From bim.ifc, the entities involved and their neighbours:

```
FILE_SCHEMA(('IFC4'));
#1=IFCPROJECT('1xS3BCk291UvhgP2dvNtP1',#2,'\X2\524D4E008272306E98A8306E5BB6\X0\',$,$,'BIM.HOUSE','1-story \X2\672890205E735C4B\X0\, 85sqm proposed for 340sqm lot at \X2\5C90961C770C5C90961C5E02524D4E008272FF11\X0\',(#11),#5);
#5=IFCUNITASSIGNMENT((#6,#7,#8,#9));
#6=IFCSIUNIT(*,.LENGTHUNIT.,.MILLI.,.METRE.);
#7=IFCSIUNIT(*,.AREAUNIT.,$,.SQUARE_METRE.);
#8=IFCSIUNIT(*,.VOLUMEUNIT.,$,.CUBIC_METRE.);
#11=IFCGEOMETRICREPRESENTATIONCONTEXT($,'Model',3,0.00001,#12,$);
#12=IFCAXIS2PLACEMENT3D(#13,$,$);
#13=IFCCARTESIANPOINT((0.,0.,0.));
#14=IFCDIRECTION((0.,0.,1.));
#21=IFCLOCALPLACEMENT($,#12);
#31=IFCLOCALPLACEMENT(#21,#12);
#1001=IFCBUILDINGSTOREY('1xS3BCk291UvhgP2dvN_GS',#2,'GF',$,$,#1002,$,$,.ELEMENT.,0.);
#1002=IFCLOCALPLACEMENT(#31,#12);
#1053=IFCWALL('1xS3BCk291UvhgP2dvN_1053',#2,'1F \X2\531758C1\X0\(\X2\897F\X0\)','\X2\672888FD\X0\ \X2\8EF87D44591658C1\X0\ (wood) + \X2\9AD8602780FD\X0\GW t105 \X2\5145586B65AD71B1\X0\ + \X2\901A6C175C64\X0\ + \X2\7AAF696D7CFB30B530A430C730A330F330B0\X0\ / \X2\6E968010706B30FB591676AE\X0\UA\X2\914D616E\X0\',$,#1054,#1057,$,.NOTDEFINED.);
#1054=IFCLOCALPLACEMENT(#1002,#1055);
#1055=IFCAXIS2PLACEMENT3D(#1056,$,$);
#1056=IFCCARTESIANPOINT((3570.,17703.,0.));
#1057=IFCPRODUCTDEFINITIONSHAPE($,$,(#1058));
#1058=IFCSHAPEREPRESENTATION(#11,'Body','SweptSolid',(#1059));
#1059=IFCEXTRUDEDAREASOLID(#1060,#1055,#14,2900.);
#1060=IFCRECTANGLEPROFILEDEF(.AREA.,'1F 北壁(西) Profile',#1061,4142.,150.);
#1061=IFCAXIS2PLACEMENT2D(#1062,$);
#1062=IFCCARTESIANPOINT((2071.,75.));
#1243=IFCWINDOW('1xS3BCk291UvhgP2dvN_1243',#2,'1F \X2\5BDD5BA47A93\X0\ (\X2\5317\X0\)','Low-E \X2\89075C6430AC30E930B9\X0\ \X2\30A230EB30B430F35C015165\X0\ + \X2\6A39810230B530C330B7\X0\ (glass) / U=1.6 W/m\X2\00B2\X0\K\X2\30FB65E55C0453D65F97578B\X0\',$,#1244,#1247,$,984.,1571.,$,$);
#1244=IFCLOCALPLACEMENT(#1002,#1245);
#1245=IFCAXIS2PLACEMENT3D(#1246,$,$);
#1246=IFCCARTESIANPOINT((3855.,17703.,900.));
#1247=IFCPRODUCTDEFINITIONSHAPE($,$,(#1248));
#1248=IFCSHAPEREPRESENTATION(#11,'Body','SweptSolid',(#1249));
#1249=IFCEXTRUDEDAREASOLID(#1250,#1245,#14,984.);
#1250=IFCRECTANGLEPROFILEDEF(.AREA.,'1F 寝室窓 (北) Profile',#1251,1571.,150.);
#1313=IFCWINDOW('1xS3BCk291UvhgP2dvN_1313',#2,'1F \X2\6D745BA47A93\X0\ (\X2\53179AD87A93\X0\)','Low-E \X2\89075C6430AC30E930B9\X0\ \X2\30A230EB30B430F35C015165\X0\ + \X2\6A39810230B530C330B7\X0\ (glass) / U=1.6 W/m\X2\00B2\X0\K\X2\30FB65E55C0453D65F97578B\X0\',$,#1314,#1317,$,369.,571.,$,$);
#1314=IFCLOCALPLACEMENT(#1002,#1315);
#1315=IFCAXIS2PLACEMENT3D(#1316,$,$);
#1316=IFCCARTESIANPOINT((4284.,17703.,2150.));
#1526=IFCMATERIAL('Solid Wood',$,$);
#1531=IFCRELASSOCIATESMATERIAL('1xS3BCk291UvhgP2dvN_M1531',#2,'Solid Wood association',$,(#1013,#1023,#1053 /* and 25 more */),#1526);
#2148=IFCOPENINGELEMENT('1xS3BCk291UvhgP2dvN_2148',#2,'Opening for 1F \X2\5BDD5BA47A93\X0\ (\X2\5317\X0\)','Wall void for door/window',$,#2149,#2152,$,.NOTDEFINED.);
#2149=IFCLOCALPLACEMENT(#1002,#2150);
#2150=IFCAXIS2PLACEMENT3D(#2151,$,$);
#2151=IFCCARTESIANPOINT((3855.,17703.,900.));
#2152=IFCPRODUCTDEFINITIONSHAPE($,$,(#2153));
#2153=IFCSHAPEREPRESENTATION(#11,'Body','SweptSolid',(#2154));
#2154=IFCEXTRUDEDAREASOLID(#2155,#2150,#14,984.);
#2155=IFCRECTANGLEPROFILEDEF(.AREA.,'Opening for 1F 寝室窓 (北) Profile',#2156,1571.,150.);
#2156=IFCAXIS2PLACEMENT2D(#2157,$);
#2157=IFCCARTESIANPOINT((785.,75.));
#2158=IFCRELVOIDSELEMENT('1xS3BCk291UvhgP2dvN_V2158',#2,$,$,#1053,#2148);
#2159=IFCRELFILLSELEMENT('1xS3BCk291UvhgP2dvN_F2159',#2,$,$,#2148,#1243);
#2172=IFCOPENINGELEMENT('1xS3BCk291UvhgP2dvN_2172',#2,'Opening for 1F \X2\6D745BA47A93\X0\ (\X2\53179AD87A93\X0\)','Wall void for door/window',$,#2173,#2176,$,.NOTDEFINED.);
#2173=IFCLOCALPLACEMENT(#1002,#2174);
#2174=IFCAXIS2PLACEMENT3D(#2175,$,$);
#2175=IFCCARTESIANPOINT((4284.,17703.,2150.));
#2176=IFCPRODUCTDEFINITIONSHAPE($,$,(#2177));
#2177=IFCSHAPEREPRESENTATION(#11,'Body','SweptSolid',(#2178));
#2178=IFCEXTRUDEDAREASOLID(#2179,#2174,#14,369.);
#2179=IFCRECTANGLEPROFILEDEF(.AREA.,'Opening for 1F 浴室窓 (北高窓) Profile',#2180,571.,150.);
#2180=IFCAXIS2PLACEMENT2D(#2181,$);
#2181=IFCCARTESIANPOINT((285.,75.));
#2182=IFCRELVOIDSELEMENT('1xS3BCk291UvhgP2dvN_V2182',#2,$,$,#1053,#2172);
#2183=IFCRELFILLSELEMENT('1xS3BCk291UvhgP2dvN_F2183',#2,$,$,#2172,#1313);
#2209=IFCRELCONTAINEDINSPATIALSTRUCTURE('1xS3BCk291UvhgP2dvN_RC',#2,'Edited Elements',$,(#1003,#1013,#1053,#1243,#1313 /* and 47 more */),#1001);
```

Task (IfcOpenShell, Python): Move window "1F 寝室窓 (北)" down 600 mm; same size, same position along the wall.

```python
import numpy as np
import ifcopenshell
import ifcopenshell.api.geometry
import ifcopenshell.util.placement
import ifcopenshell.util.unit

model = ifcopenshell.open("bim.ifc")
unit_scale = ifcopenshell.util.unit.calculate_unit_scale(model)

window = model.by_id(1243)
opening = window.FillsVoids[0].RelatingOpeningElement
dz = -0.6 / unit_scale

shift = np.array([0.0, 0.0, dz])
# The window is not placed relative to its opening, so move both.
for product in (opening, window):
    matrix = ifcopenshell.util.placement.get_local_placement(product.ObjectPlacement)
    matrix[:3, 3] += shift
    ifcopenshell.api.geometry.edit_object_placement(model, product=product, matrix=matrix, is_si=False)

print(f"moved by {dz * unit_scale:+.3f} m")

model.write("bim_edited.ifc")
```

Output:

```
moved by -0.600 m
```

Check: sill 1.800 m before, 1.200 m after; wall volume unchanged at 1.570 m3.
